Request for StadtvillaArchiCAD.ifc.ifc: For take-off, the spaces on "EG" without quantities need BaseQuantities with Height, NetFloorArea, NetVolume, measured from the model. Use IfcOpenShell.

First a look at what the model holds.

```python
import ifcopenshell
import ifcopenshell.util.element
import ifcopenshell.util.unit

model = ifcopenshell.open("StadtvillaArchiCAD.ifc.ifc")
print(model.schema)
for unit_type in ("LENGTHUNIT", "AREAUNIT", "VOLUMEUNIT"):
    print(unit_type, ifcopenshell.util.unit.calculate_unit_scale(model, unit_type))
storey = next(s for s in model.by_type("IfcBuildingStorey") if s.Name == "EG")
spaces = [e for e in ifcopenshell.util.element.get_decomposition(storey) if e.is_a("IfcSpace")]
for e in sorted(spaces, key=lambda e: e.id()):
    print(e.id(), e.is_a(), e.Name, list(ifcopenshell.util.element.get_psets(e, qtos_only=True)), sep=" | ")
```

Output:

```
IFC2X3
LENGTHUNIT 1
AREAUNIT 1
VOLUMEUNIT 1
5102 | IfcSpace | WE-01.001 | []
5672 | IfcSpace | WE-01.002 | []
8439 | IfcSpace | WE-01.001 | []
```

```python
import ifcopenshell
import ifcopenshell.api.pset
import ifcopenshell.geom
import ifcopenshell.util.element
import ifcopenshell.util.shape
import ifcopenshell.util.unit

model = ifcopenshell.open("StadtvillaArchiCAD.ifc.ifc")
unit_scale = ifcopenshell.util.unit.calculate_unit_scale(model)
area_scale = ifcopenshell.util.unit.calculate_unit_scale(model, "AREAUNIT")
volume_scale = ifcopenshell.util.unit.calculate_unit_scale(model, "VOLUMEUNIT")
settings = ifcopenshell.geom.settings()

storey = next(s for s in model.by_type("IfcBuildingStorey") if s.Name == "EG")
spaces = [e for e in ifcopenshell.util.element.get_decomposition(storey) if e.is_a("IfcSpace")]

for e in sorted(spaces, key=lambda e: e.id()):
    if ifcopenshell.util.element.get_psets(e, qtos_only=True, should_inherit=False):
        continue
    # Geometry comes back in metres, in the element's own axes.
    shape = ifcopenshell.geom.create_shape(settings, e)
    values = {
        "Height": ifcopenshell.util.shape.get_z(shape.geometry) / unit_scale,
        "NetFloorArea": ifcopenshell.util.shape.get_footprint_area(shape.geometry) / area_scale,
        "NetVolume": ifcopenshell.util.shape.get_volume(shape.geometry) / volume_scale,
    }
    qto = ifcopenshell.api.pset.add_qto(model, product=e, name="BaseQuantities")
    ifcopenshell.api.pset.edit_qto(model, qto=qto, properties=values)
    print(e.id(), {k: round(v, 3) for k, v in values.items()})

model.write("StadtvillaArchiCAD.ifc_edited.ifc")
```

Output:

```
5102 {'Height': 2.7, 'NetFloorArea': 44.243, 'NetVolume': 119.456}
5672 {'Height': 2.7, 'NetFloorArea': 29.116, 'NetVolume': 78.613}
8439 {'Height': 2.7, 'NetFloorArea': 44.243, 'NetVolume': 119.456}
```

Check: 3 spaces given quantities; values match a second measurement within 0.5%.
